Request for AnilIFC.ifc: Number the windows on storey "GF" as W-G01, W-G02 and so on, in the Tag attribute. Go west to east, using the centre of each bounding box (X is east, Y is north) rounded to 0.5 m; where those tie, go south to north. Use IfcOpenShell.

First a look at what the model holds.

```python
import ifcopenshell
import ifcopenshell.util.element
import ifcopenshell.util.placement

model = ifcopenshell.open("AnilIFC.ifc")
print(model.schema)
storey = next(s for s in model.by_type("IfcBuildingStorey") if s.Name == "GF")
windows = [e for e in ifcopenshell.util.element.get_decomposition(storey) if e.is_a("IfcWindow")]
for e in sorted(windows, key=lambda e: e.id()):
    origin = ifcopenshell.util.placement.get_local_placement(e.ObjectPlacement)[:3, 3]
    print(e.id(), e.Tag, e.Name, origin.round(2) + 0.0, sep=" | ")
```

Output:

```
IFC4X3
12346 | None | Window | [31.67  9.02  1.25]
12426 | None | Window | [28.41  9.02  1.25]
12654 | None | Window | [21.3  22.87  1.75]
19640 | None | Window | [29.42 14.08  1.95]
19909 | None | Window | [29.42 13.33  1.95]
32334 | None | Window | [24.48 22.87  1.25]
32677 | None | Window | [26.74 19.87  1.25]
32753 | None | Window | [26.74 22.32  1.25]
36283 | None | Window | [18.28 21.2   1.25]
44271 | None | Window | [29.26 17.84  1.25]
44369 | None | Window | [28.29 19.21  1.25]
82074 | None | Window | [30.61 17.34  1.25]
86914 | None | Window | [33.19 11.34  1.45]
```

```python
import ifcopenshell
import ifcopenshell.geom
import ifcopenshell.util.element
import ifcopenshell.util.shape

model = ifcopenshell.open("AnilIFC.ifc")
settings = ifcopenshell.geom.settings()
settings.set("use-world-coords", True)


def centre(element):
    shape = ifcopenshell.geom.create_shape(settings, element)
    return ifcopenshell.util.shape.get_bbox_centroid(shape.geometry)


storey = next(s for s in model.by_type("IfcBuildingStorey") if s.Name == "GF")
windows = [e for e in ifcopenshell.util.element.get_decomposition(storey) if e.is_a("IfcWindow")]

# Insertion points can sit at a corner or the storey origin, so sort by the geometry (in metres).
centres = {e: centre(e) for e in windows}
windows.sort(key=lambda e: (round(centres[e][0] / 0.5), centres[e][1]))

for i, e in enumerate(windows, start=1):
    number = f"W-G{i:02d}"
    e.Tag = number
    print(e.id(), number)

model.write("AnilIFC_edited.ifc")
```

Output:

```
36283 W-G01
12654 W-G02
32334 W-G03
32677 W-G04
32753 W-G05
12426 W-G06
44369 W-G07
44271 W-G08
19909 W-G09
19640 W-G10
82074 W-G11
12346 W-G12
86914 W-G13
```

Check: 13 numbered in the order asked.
